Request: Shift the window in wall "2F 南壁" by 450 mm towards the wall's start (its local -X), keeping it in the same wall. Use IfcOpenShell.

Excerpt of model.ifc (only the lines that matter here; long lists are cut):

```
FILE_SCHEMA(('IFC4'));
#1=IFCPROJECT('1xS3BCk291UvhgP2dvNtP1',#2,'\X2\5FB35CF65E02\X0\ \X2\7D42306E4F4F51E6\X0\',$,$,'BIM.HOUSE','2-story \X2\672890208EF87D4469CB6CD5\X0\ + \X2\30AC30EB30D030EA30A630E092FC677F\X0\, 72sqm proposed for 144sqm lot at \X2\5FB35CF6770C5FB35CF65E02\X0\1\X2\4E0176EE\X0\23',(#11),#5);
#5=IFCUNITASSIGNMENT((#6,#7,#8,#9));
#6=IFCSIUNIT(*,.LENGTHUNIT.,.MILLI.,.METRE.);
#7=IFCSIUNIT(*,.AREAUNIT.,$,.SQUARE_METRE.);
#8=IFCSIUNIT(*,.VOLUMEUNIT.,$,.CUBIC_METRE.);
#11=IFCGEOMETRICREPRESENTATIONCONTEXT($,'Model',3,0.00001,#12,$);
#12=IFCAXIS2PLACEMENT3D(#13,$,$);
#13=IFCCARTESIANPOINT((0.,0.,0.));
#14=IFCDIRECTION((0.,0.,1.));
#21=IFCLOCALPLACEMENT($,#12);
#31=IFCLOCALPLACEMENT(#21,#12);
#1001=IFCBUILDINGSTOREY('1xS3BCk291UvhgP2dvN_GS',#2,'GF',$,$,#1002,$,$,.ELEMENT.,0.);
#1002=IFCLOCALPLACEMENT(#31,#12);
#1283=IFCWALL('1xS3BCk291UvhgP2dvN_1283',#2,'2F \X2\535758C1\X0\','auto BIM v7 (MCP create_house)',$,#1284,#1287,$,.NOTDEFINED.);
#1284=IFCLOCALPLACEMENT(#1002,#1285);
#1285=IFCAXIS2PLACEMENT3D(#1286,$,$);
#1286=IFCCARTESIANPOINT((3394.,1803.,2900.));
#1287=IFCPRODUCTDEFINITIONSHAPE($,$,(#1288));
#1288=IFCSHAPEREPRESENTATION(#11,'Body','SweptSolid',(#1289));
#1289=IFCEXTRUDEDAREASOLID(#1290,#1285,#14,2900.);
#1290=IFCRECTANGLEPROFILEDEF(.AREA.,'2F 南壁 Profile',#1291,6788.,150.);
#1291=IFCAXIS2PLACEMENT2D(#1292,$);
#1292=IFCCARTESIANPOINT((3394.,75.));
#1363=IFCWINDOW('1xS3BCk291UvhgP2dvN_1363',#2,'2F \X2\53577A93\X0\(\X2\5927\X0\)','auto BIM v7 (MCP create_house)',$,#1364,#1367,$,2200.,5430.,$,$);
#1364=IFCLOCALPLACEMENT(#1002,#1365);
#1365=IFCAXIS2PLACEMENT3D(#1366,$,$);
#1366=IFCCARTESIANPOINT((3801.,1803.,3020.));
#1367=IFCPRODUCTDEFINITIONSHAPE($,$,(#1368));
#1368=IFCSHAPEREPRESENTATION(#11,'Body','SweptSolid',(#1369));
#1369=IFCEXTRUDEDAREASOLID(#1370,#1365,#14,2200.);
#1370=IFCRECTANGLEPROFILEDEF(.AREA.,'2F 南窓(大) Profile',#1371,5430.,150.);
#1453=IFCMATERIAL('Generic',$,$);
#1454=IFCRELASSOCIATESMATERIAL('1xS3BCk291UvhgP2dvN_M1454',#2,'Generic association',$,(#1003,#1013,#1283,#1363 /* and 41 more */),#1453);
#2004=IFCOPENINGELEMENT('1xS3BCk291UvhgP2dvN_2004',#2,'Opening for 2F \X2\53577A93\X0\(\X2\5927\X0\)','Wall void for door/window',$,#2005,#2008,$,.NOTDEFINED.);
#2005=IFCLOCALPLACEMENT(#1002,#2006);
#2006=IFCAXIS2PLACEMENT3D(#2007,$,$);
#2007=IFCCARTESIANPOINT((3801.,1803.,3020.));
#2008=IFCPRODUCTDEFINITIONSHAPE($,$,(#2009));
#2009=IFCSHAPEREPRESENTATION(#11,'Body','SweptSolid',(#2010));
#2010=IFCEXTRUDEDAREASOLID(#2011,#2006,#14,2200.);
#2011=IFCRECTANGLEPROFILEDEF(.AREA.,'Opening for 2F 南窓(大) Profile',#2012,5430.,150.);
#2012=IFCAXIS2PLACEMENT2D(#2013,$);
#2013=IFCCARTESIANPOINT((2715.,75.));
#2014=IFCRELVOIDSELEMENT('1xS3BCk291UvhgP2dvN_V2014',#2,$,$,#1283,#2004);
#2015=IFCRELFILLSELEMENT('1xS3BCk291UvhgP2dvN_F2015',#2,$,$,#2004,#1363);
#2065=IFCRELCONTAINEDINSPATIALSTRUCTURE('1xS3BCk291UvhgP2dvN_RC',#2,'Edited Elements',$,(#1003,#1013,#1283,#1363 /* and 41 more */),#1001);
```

```python
import ifcopenshell
import ifcopenshell.api.geometry
import ifcopenshell.util.placement
import ifcopenshell.util.unit

model = ifcopenshell.open("model.ifc")
unit_scale = ifcopenshell.util.unit.calculate_unit_scale(model)

window = model.by_guid("1xS3BCk291UvhgP2dvN_1363")
opening = window.FillsVoids[0].RelatingOpeningElement
wall = opening.VoidsElements[0].RelatingBuildingElement

wall_matrix = ifcopenshell.util.placement.get_local_placement(wall.ObjectPlacement)
shift = wall_matrix[:3, 0] * -0.45 / unit_scale
before = ifcopenshell.util.placement.get_local_placement(window.ObjectPlacement)[:3, 3].copy()

# The window is not placed relative to its opening, so move both.
for product in (opening, window):
    matrix = ifcopenshell.util.placement.get_local_placement(product.ObjectPlacement)
    matrix[:3, 3] += shift
    ifcopenshell.api.geometry.edit_object_placement(model, product=product, matrix=matrix, is_si=False)

after = ifcopenshell.util.placement.get_local_placement(window.ObjectPlacement)[:3, 3]
print("window moved by", (after - before).round(3) + 0.0)

model.write("model-out.ifc")
```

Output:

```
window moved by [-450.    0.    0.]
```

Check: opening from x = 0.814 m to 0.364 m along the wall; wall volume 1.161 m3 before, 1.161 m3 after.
